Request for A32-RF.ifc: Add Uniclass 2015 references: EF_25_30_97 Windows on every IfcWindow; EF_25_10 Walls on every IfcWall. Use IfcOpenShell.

First a look at what the model holds.

```python
import ifcopenshell

model = ifcopenshell.open("A32-RF.ifc")
print(model.schema)
print("classifications:", [c.Name for c in model.by_type("IfcClassification")])
for ifc_class in ("IfcDoor", "IfcRoof", "IfcStair", "IfcWall", "IfcWindow"):
    print(ifc_class, len(model.by_type(ifc_class)))
```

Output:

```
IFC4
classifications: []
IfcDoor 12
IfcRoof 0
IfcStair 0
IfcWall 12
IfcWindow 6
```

```python
import ifcopenshell
import ifcopenshell.api.classification

model = ifcopenshell.open("A32-RF.ifc")

system = ifcopenshell.api.classification.add_classification(model, classification="Uniclass 2015")

codes = {
    "IfcWindow": ("EF_25_30_97", "Windows"),
    "IfcWall": ("EF_25_10", "Walls"),
}
for ifc_class, (code, name) in codes.items():
    products = model.by_type(ifc_class)
    ifcopenshell.api.classification.add_reference(
        model, products=products, classification=system, identification=code, name=name
    )
    print(code, len(products))

model.write("A32-RF_updated.ifc")
```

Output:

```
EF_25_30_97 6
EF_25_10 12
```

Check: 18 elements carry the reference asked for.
